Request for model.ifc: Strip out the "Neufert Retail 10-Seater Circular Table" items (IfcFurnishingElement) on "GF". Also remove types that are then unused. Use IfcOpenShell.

First a look at what the model holds.

```python
import ifcopenshell
import ifcopenshell.util.element

model = ifcopenshell.open("model.ifc")
print(model.schema)
storey = next(s for s in model.by_type("IfcBuildingStorey") if s.Name == "GF")
furniture = [e for e in ifcopenshell.util.element.get_decomposition(storey) if e.is_a("IfcFurnishingElement")]
seen = {}
for e in furniture:
    element_type = ifcopenshell.util.element.get_type(e)
    name = element_type.Name if element_type not in (None, e) else None
    seen[name] = seen.get(name, 0) + 1
for name, count in sorted(seen.items(), key=str):
    print(count, "x", name)
```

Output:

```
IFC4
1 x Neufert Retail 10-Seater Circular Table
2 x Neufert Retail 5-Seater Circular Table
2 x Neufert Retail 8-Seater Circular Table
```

```python
import ifcopenshell
import ifcopenshell.api.root
import ifcopenshell.util.element

model = ifcopenshell.open("model.ifc")

storey = next(s for s in model.by_type("IfcBuildingStorey") if s.Name == "GF")
furniture = [e for e in ifcopenshell.util.element.get_decomposition(storey) if e.is_a("IfcFurnishingElement")]
targets = [e for e in furniture if (t := ifcopenshell.util.element.get_type(e)) not in (None, e) and t.Name == "Neufert Retail 10-Seater Circular Table"]
types = {ifcopenshell.util.element.get_type(e) for e in targets} - {None, *targets}

for e in targets:
    ifcopenshell.api.root.remove_product(model, product=e)
print(len(targets), "removed")

unused = [t for t in types if not ifcopenshell.util.element.get_types(t)]
for t in unused:
    ifcopenshell.api.root.remove_product(model, product=t)
print(len(unused), "unused types removed")

model.write("model_edited.ifc")
```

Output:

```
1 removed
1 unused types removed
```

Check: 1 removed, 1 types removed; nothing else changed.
